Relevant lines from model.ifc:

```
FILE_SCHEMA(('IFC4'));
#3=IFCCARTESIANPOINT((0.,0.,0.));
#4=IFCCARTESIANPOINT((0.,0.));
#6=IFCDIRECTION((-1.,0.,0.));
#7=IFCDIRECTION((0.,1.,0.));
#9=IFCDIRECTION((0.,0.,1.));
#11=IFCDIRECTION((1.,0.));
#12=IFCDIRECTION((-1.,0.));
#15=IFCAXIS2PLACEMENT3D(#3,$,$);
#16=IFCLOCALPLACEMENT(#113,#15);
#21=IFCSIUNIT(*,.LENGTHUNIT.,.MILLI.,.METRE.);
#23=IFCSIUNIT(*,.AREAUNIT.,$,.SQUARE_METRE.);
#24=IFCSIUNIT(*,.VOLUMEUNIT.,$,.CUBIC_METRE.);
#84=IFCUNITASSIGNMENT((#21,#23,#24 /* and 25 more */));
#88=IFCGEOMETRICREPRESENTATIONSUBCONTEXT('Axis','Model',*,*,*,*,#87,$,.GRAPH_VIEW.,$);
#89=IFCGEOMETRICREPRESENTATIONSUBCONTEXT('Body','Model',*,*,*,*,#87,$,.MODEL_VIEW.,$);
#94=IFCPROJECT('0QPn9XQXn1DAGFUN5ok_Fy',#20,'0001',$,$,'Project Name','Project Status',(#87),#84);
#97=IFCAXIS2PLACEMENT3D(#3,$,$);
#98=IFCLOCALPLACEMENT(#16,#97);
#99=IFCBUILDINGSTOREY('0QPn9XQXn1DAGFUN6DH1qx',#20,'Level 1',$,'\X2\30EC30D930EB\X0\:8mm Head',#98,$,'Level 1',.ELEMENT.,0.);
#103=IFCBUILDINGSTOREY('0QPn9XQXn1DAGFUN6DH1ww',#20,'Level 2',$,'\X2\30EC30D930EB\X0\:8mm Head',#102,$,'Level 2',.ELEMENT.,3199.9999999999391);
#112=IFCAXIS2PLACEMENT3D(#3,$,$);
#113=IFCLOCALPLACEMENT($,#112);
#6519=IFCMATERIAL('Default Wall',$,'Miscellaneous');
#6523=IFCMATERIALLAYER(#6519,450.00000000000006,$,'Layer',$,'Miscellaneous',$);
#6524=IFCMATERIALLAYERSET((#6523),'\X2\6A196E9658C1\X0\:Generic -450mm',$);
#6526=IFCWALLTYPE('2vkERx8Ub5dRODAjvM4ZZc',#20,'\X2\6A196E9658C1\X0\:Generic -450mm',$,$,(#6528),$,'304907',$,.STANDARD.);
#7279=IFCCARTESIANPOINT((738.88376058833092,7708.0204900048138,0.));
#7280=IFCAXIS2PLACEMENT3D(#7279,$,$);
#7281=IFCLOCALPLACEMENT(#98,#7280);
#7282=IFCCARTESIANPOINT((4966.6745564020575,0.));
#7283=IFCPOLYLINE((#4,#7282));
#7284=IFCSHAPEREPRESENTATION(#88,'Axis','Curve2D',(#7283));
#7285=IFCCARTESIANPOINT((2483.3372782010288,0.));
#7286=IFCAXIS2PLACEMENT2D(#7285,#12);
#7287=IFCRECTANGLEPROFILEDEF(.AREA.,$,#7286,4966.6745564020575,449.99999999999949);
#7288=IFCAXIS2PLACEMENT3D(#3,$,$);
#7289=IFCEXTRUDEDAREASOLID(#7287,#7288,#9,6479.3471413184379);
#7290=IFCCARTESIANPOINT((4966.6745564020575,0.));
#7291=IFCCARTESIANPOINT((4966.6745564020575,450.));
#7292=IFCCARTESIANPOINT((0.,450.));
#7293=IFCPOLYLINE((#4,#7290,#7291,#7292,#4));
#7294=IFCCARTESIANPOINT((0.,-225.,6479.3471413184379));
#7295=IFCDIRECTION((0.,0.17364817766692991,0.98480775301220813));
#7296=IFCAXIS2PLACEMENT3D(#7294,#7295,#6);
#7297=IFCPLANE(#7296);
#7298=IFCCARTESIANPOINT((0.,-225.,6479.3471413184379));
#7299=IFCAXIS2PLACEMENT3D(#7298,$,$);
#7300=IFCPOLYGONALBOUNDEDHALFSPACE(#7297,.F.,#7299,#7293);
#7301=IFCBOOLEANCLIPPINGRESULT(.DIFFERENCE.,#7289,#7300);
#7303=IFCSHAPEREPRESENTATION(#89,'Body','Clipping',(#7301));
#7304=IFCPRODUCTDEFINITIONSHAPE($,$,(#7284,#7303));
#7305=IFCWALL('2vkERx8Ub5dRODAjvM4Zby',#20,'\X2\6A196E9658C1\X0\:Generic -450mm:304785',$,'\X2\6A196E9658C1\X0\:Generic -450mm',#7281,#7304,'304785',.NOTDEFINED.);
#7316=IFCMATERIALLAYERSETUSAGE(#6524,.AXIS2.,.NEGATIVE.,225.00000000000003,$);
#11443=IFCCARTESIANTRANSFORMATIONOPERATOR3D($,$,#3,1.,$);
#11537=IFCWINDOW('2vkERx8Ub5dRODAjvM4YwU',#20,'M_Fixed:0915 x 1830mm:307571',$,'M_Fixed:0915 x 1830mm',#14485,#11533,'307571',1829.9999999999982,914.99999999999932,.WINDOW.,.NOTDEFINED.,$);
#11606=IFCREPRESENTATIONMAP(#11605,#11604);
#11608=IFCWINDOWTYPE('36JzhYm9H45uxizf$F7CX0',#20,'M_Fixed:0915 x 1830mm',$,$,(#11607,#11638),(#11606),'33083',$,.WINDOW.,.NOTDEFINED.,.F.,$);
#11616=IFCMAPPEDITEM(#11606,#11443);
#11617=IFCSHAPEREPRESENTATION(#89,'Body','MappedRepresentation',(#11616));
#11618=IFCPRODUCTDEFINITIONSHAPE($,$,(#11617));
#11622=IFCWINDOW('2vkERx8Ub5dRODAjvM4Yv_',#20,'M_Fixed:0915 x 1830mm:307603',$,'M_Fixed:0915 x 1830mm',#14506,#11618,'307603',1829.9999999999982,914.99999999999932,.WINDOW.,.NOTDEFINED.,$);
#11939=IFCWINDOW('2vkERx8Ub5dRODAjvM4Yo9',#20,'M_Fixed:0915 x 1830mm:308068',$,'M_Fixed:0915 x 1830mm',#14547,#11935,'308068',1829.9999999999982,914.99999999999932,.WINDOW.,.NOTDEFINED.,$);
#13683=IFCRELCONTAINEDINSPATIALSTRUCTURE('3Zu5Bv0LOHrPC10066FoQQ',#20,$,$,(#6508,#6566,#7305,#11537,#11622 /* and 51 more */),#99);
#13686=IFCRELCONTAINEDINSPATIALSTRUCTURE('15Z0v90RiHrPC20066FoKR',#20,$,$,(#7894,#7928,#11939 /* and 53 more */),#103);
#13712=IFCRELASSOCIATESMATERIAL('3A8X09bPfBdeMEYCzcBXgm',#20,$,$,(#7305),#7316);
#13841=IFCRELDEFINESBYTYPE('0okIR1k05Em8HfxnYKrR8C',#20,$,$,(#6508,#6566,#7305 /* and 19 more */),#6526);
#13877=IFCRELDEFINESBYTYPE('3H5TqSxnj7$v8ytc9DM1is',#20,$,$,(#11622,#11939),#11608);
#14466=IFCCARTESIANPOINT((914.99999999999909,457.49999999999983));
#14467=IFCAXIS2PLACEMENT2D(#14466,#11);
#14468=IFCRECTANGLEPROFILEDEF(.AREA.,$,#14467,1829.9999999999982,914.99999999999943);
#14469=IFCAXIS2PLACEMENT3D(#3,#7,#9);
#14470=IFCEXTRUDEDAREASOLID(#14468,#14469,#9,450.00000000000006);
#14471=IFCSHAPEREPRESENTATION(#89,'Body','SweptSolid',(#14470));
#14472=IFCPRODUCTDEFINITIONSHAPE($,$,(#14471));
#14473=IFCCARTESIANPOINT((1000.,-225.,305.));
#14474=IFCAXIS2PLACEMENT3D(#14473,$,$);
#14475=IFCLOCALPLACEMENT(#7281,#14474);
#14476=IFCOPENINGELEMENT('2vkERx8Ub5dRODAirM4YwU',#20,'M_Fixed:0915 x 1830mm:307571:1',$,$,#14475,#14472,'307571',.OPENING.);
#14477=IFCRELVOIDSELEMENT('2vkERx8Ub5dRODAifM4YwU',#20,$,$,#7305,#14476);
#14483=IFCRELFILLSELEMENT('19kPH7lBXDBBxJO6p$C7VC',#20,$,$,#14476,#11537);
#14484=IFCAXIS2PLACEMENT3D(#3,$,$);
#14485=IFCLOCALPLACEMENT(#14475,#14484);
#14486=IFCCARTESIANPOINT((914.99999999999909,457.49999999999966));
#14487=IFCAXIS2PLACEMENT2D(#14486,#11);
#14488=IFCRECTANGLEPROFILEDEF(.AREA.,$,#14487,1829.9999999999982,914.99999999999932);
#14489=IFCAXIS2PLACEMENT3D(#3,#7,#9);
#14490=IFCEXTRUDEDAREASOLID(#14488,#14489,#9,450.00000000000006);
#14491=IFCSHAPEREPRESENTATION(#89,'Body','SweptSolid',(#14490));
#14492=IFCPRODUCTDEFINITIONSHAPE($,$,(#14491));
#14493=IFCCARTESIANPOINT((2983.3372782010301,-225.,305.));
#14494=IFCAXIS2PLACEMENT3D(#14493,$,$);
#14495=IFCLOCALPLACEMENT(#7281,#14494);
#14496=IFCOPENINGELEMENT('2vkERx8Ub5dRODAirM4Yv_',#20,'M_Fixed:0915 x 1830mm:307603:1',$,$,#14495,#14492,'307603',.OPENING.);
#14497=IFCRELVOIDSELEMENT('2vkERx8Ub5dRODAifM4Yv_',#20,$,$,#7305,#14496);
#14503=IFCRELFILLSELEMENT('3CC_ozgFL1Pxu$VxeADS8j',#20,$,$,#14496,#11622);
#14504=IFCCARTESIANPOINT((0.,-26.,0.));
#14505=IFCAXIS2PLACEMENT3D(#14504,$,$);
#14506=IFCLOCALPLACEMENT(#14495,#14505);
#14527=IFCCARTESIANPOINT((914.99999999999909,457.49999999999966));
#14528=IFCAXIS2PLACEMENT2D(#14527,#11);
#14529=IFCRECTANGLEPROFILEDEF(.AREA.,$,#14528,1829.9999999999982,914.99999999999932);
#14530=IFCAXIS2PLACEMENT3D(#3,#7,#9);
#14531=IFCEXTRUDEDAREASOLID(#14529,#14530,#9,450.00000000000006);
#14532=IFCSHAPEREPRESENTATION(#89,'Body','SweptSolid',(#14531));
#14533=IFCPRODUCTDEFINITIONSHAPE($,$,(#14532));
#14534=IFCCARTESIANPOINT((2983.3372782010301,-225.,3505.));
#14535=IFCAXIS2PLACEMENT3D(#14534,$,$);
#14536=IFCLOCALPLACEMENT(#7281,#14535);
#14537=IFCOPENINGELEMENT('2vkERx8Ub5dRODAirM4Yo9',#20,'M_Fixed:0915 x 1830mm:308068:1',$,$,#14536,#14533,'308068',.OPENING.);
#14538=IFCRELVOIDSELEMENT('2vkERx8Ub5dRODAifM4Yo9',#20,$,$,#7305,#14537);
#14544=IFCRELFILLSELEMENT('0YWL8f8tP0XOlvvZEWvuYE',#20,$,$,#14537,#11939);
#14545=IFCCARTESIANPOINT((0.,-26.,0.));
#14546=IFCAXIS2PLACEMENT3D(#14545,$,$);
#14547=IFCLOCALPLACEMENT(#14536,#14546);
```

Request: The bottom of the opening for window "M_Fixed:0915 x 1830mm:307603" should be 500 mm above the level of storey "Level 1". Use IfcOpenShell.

```python
import numpy as np
import ifcopenshell
import ifcopenshell.api.geometry
import ifcopenshell.geom
import ifcopenshell.util.element
import ifcopenshell.util.placement
import ifcopenshell.util.shape
import ifcopenshell.util.unit

model = ifcopenshell.open("model.ifc")
unit_scale = ifcopenshell.util.unit.calculate_unit_scale(model)

window = model.by_guid("2vkERx8Ub5dRODAjvM4Yv_")
opening = window.FillsVoids[0].RelatingOpeningElement
storey = ifcopenshell.util.element.get_container(window, ifc_class="IfcBuildingStorey")
level = ifcopenshell.util.placement.get_local_placement(storey.ObjectPlacement)[2, 3]

# The opening's origin need not be at the sill, so measure its lowest point.
shape = ifcopenshell.geom.create_shape(ifcopenshell.geom.settings(), opening)
bottom = ifcopenshell.util.shape.get_shape_bottom_elevation(shape, shape.geometry) / unit_scale
dz = level + 0.5 / unit_scale - bottom

shift = np.array([0.0, 0.0, dz])
# The window is placed relative to its opening, so it follows when the opening moves.
matrix = ifcopenshell.util.placement.get_local_placement(opening.ObjectPlacement)
matrix[:3, 3] += shift
ifcopenshell.api.geometry.edit_object_placement(
    model, product=opening, matrix=matrix, is_si=False, should_transform_children=True
)

print(f"moved by {dz * unit_scale:+.3f} m")

model.write("model_edited.ifc")
```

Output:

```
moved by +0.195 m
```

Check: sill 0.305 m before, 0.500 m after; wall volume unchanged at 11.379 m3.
